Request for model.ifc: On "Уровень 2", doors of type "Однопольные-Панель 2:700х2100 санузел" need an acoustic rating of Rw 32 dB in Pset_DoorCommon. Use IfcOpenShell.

First a look at what the model holds.

```python
import ifcopenshell
import ifcopenshell.util.element

model = ifcopenshell.open("model.ifc")
print(model.schema)
storey = next(s for s in model.by_type("IfcBuildingStorey") if s.Name == "Уровень 2")
doors = [e for e in ifcopenshell.util.element.get_decomposition(storey) if e.is_a("IfcDoor")]
seen = {}
for e in doors:
    element_type = ifcopenshell.util.element.get_type(e)
    key = (element_type.Name if element_type != e and element_type else None, ifcopenshell.util.element.get_pset(e, "Pset_DoorCommon", "AcousticRating"))
    seen[key] = seen.get(key, 0) + 1
for (name, value), count in sorted(seen.items(), key=str):
    print(count, "x", name, "|", value)
```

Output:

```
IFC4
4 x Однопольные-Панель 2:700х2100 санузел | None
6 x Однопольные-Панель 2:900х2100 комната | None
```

```python
import ifcopenshell
import ifcopenshell.api.pset
import ifcopenshell.util.element

model = ifcopenshell.open("model.ifc")

storey = next(s for s in model.by_type("IfcBuildingStorey") if s.Name == "Уровень 2")
doors = [e for e in ifcopenshell.util.element.get_decomposition(storey) if e.is_a("IfcDoor")]

count = 0
for e in doors:
    element_type = ifcopenshell.util.element.get_type(e)
    if element_type in (None, e) or element_type.Name != "Однопольные-Панель 2:700х2100 санузел":
        continue
    # add_pset returns the element's existing set when there is one.
    pset = ifcopenshell.api.pset.add_pset(model, product=e, name="Pset_DoorCommon")
    ifcopenshell.api.pset.edit_pset(model, pset=pset, properties={"AcousticRating": "Rw 32 dB"})
    count += 1

print(count, "doors updated")

model.write("model-out.ifc")
```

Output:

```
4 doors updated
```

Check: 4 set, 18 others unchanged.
